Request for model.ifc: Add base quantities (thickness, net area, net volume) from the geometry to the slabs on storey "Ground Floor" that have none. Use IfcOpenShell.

First a look at what the model holds.

```python
import ifcopenshell
import ifcopenshell.util.element
import ifcopenshell.util.unit

model = ifcopenshell.open("model.ifc")
print(model.schema)
for unit_type in ("LENGTHUNIT", "AREAUNIT", "VOLUMEUNIT"):
    print(unit_type, ifcopenshell.util.unit.calculate_unit_scale(model, unit_type))
storey = next(s for s in model.by_type("IfcBuildingStorey") if s.Name == "Ground Floor")
slabs = [e for e in ifcopenshell.util.element.get_decomposition(storey) if e.is_a("IfcSlab")]
for e in sorted(slabs, key=lambda e: e.id()):
    print(e.id(), e.is_a(), e.Name, list(ifcopenshell.util.element.get_psets(e, qtos_only=True)), sep=" | ")
```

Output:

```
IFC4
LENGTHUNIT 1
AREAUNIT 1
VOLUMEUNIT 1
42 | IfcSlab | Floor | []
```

```python
import ifcopenshell
import ifcopenshell.api.pset
import ifcopenshell.geom
import ifcopenshell.util.element
import ifcopenshell.util.shape
import ifcopenshell.util.unit

model = ifcopenshell.open("model.ifc")
unit_scale = ifcopenshell.util.unit.calculate_unit_scale(model)
area_scale = ifcopenshell.util.unit.calculate_unit_scale(model, "AREAUNIT")
volume_scale = ifcopenshell.util.unit.calculate_unit_scale(model, "VOLUMEUNIT")
settings = ifcopenshell.geom.settings()

storey = next(s for s in model.by_type("IfcBuildingStorey") if s.Name == "Ground Floor")
slabs = [e for e in ifcopenshell.util.element.get_decomposition(storey) if e.is_a("IfcSlab")]

for e in sorted(slabs, key=lambda e: e.id()):
    if ifcopenshell.util.element.get_psets(e, qtos_only=True, should_inherit=False):
        continue
    # Geometry comes back in metres, in the element's own axes.
    shape = ifcopenshell.geom.create_shape(settings, e)
    values = {
        "Width": ifcopenshell.util.shape.get_z(shape.geometry) / unit_scale,
        "NetArea": ifcopenshell.util.shape.get_footprint_area(shape.geometry) / area_scale,
        "NetVolume": ifcopenshell.util.shape.get_volume(shape.geometry) / volume_scale,
    }
    qto = ifcopenshell.api.pset.add_qto(model, product=e, name="Qto_SlabBaseQuantities")
    ifcopenshell.api.pset.edit_qto(model, qto=qto, properties=values)
    print(e.id(), {k: round(v, 3) for k, v in values.items()})

model.write("model_v2.ifc")
```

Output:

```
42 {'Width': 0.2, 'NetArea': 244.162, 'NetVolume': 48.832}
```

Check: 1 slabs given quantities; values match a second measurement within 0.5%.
